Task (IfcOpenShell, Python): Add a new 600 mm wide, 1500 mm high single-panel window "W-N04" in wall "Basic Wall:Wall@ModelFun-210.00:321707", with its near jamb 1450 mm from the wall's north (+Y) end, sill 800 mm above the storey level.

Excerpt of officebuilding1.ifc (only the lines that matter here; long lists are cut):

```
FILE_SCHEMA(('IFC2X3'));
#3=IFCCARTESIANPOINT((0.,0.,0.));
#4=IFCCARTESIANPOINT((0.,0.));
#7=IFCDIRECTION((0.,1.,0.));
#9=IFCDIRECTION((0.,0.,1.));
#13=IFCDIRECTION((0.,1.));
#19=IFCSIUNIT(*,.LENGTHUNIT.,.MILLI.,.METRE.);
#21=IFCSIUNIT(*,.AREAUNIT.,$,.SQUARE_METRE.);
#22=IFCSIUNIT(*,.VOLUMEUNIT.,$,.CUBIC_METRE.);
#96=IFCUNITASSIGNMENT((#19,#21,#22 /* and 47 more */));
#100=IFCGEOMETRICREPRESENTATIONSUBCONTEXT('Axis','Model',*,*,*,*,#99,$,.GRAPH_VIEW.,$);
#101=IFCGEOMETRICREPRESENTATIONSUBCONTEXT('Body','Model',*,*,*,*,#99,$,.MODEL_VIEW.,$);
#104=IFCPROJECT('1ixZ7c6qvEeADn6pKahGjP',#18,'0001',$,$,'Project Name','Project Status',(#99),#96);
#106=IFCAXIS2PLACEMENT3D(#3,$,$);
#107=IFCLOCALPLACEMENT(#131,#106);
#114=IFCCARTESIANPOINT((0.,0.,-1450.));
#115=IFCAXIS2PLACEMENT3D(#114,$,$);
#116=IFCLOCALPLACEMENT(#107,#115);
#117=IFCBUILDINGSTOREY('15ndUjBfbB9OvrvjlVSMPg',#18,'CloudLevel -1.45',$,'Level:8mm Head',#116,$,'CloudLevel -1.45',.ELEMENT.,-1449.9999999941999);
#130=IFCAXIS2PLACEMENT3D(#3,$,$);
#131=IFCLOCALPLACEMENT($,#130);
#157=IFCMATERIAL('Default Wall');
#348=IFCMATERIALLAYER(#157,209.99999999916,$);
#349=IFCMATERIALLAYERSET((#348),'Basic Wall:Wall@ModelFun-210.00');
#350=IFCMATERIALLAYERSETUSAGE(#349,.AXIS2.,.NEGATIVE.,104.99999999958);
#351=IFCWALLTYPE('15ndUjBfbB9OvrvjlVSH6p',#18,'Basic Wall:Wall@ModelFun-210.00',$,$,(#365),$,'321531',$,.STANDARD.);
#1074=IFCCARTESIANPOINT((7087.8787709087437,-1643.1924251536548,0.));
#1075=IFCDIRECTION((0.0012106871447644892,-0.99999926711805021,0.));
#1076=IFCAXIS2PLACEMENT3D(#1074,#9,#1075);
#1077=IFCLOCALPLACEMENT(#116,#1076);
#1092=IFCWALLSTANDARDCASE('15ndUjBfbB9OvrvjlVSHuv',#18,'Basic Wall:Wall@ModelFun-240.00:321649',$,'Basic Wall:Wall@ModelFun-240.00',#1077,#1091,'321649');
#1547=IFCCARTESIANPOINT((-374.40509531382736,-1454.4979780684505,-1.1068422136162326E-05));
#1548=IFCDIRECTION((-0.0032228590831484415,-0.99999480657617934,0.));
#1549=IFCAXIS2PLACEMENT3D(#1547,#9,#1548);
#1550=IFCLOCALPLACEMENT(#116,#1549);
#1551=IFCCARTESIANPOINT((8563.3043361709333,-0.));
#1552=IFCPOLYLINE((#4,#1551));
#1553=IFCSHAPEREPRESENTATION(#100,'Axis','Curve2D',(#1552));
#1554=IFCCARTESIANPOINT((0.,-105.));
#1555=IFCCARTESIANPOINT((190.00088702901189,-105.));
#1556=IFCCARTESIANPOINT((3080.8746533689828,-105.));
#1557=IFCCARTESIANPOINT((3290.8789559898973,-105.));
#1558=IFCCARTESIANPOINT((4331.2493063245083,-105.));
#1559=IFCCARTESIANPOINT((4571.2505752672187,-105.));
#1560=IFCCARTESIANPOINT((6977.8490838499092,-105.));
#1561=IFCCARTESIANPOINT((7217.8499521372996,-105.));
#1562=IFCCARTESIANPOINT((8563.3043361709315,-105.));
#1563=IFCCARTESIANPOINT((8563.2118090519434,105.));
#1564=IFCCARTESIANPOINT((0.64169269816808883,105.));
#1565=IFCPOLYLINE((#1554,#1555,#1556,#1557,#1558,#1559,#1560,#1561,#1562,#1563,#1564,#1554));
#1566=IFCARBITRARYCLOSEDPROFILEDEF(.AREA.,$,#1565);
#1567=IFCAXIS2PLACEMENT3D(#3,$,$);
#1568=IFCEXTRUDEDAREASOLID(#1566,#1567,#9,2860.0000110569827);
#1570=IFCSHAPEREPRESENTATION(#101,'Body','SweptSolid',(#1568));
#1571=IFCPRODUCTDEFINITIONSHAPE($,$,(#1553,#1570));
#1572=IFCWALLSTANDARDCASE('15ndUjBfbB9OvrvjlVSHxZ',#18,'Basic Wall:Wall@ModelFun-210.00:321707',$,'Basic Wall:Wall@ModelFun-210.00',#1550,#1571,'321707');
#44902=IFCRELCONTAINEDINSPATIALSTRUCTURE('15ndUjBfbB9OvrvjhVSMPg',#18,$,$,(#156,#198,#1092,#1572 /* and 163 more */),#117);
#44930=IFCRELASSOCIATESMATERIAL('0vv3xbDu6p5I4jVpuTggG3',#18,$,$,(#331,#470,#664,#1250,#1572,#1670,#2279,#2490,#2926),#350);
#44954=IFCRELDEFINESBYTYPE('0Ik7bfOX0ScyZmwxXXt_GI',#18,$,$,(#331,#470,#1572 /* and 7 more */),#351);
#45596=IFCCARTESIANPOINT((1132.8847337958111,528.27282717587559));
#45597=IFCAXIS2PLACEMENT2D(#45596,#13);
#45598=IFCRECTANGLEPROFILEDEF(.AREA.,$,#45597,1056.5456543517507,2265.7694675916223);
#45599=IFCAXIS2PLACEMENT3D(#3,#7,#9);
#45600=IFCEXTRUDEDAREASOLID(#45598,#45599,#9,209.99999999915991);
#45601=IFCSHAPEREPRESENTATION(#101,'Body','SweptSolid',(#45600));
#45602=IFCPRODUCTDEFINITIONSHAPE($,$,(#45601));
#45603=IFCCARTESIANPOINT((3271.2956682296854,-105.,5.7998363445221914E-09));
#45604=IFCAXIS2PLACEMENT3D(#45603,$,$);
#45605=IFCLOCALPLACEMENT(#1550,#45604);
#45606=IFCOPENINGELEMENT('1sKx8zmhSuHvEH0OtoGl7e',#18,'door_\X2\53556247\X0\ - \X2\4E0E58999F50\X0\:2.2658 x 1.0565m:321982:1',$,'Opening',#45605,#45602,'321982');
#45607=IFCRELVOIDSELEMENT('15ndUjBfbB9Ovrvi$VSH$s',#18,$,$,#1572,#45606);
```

```python
import numpy as np
import ifcopenshell
import ifcopenshell.api.feature
import ifcopenshell.api.geometry
import ifcopenshell.api.root
import ifcopenshell.api.spatial
import ifcopenshell.api.type
import ifcopenshell.geom
import ifcopenshell.util.element
import ifcopenshell.util.placement
import ifcopenshell.util.representation
import ifcopenshell.util.shape
import ifcopenshell.util.unit

model = ifcopenshell.open("officebuilding1.ifc")
unit_scale = ifcopenshell.util.unit.calculate_unit_scale(model)
settings = ifcopenshell.geom.settings()


def volume(element):
    """Net volume in cubic metres, openings subtracted."""
    shape = ifcopenshell.geom.create_shape(settings, element)
    return ifcopenshell.util.shape.get_volume(shape.geometry)


wall = model.by_id(1572)
storey = ifcopenshell.util.element.get_container(wall, ifc_class="IfcBuildingStorey")
context = ifcopenshell.util.representation.get_context(model, "Model", "Body", "MODEL_VIEW")
before = volume(wall)

width, height, from_end, sill = 0.6, 1.5, 1.45, 0.8  # metres

# The wall runs along its own X axis, and the end named is its -X end.
wall_shape = ifcopenshell.geom.create_shape(settings, wall)
x, y, z = ifcopenshell.util.shape.get_vertices(wall_shape.geometry).T
start = x.min() + from_end
face, thickness = float(y.min()), float(y.max() - y.min())
wall_matrix = ifcopenshell.util.placement.get_local_placement(wall.ObjectPlacement)
level = ifcopenshell.util.placement.get_local_placement(storey.ObjectPlacement)[2, 3]


def in_wall(x, y):
    """Placement at x, y metres in the wall's axes, at sill height."""
    matrix = wall_matrix.copy()
    matrix[:, 3] = wall_matrix @ np.array([x / unit_scale, y / unit_scale, 0.0, 1.0])
    matrix[2, 3] = level + sill / unit_scale
    return matrix


# Opening: a box that overshoots both wall faces by 50 mm.
opening = ifcopenshell.api.root.create_entity(model, ifc_class="IfcOpeningElement")
box = ifcopenshell.api.geometry.add_wall_representation(
    model, context=context, length=width, height=height, thickness=thickness + 0.1
)
ifcopenshell.api.geometry.assign_representation(model, product=opening, representation=box)
ifcopenshell.api.geometry.edit_object_placement(model, product=opening, matrix=in_wall(start, face - 0.05), is_si=False)
ifcopenshell.api.feature.add_feature(model, feature=opening, element=wall)

window = ifcopenshell.api.root.create_entity(model, ifc_class="IfcWindow", name="W-N04")
window.OverallWidth, window.OverallHeight = width / unit_scale, height / unit_scale
body = ifcopenshell.api.geometry.add_window_representation(
    model,
    context=context,
    overall_width=window.OverallWidth,
    overall_height=window.OverallHeight,
    partition_type="SINGLE_PANEL",
)
ifcopenshell.api.geometry.assign_representation(model, product=window, representation=body)
ifcopenshell.api.spatial.assign_container(model, products=[window], relating_structure=storey)
fills = ifcopenshell.api.feature.add_filling(model, opening=opening, element=window)
fills.OwnerHistory = window.OwnerHistory  # required in IFC2X3

# IFC2X3 keeps the operation on the window style.
style = ifcopenshell.api.root.create_entity(model, ifc_class="IfcWindowStyle", name="W-N04")
style.OperationType, style.ConstructionType = "SINGLE_PANEL", "NOTDEFINED"
style.ParameterTakesPrecedence = style.Sizeable = False
ifcopenshell.api.type.assign_type(model, related_objects=[window], relating_type=style)

# Centre the window in the wall's thickness.
ifcopenshell.api.geometry.edit_object_placement(model, product=window, matrix=in_wall(start, face), is_si=False)
window_shape = ifcopenshell.geom.create_shape(settings, window)
depth = ifcopenshell.util.shape.get_vertices(window_shape.geometry)[:, 1]
offset = face + thickness / 2 - (depth.min() + depth.max()) / 2
ifcopenshell.api.geometry.edit_object_placement(model, product=window, matrix=in_wall(start, offset), is_si=False)

after = volume(wall)

print(f"wall volume {before:.3f} -> {after:.3f} m3")

model.write("officebuilding1-out.ifc")
```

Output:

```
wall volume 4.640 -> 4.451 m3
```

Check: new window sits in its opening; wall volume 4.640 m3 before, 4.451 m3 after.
